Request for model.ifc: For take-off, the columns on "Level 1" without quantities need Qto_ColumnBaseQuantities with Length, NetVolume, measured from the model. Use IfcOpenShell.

First a look at what the model holds.

```python
import ifcopenshell
import ifcopenshell.util.element
import ifcopenshell.util.unit

model = ifcopenshell.open("model.ifc")
print(model.schema)
for unit_type in ("LENGTHUNIT", "AREAUNIT", "VOLUMEUNIT"):
    print(unit_type, ifcopenshell.util.unit.calculate_unit_scale(model, unit_type))
storey = next(s for s in model.by_type("IfcBuildingStorey") if s.Name == "Level 1")
columns = [e for e in ifcopenshell.util.element.get_decomposition(storey) if e.is_a("IfcColumn")]
for e in sorted(columns, key=lambda e: e.id()):
    print(e.id(), e.is_a(), e.Name, list(ifcopenshell.util.element.get_psets(e, qtos_only=True)), sep=" | ")
```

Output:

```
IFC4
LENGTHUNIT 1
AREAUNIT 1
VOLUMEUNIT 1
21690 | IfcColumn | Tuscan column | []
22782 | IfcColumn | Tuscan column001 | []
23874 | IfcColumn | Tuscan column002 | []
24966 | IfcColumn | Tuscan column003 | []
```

```python
import ifcopenshell
import ifcopenshell.api.pset
import ifcopenshell.geom
import ifcopenshell.util.element
import ifcopenshell.util.shape
import ifcopenshell.util.unit

model = ifcopenshell.open("model.ifc")
unit_scale = ifcopenshell.util.unit.calculate_unit_scale(model)
volume_scale = ifcopenshell.util.unit.calculate_unit_scale(model, "VOLUMEUNIT")
settings = ifcopenshell.geom.settings()

storey = next(s for s in model.by_type("IfcBuildingStorey") if s.Name == "Level 1")
columns = [e for e in ifcopenshell.util.element.get_decomposition(storey) if e.is_a("IfcColumn")]

for e in sorted(columns, key=lambda e: e.id()):
    if ifcopenshell.util.element.get_psets(e, qtos_only=True, should_inherit=False):
        continue
    # Geometry comes back in metres, in the element's own axes.
    shape = ifcopenshell.geom.create_shape(settings, e)
    values = {
        "Length": ifcopenshell.util.shape.get_z(shape.geometry) / unit_scale,
        "NetVolume": ifcopenshell.util.shape.get_volume(shape.geometry) / volume_scale,
    }
    qto = ifcopenshell.api.pset.add_qto(model, product=e, name="Qto_ColumnBaseQuantities")
    ifcopenshell.api.pset.edit_qto(model, qto=qto, properties=values)
    print(e.id(), {k: round(v, 3) for k, v in values.items()})

model.write("model-out.ifc")
```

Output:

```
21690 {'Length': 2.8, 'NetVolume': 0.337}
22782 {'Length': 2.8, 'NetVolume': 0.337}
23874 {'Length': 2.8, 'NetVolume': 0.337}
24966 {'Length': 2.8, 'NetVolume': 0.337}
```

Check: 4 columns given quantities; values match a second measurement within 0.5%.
